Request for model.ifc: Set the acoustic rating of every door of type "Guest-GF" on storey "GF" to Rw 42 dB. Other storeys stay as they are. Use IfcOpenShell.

First a look at what the model holds.

```python
import ifcopenshell
import ifcopenshell.util.element

model = ifcopenshell.open("model.ifc")
print(model.schema)
storey = next(s for s in model.by_type("IfcBuildingStorey") if s.Name == "GF")
doors = [e for e in ifcopenshell.util.element.get_decomposition(storey) if e.is_a("IfcDoor")]
seen = {}
for e in doors:
    element_type = ifcopenshell.util.element.get_type(e)
    key = (element_type.Name if element_type != e and element_type else None, ifcopenshell.util.element.get_pset(e, "Pset_DoorCommon", "AcousticRating"))
    seen[key] = seen.get(key, 0) + 1
for (name, value), count in sorted(seen.items(), key=str):
    print(count, "x", name, "|", value)
```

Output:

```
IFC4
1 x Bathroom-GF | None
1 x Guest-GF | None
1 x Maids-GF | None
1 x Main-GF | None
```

```python
import ifcopenshell
import ifcopenshell.api.pset
import ifcopenshell.util.element

model = ifcopenshell.open("model.ifc")

storey = next(s for s in model.by_type("IfcBuildingStorey") if s.Name == "GF")
doors = [e for e in ifcopenshell.util.element.get_decomposition(storey) if e.is_a("IfcDoor")]

count = 0
for e in doors:
    element_type = ifcopenshell.util.element.get_type(e)
    if element_type in (None, e) or element_type.Name != "Guest-GF":
        continue
    # add_pset returns the element's existing set when there is one.
    pset = ifcopenshell.api.pset.add_pset(model, product=e, name="Pset_DoorCommon")
    ifcopenshell.api.pset.edit_pset(model, pset=pset, properties={"AcousticRating": "Rw 42 dB"})
    count += 1

print(count, "doors updated")

model.write("model_rev.ifc")
```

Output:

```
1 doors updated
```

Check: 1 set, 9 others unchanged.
